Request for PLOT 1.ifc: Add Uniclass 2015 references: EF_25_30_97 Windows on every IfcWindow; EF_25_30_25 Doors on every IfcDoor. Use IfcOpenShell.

First a look at what the model holds.

```python
import ifcopenshell

model = ifcopenshell.open("PLOT 1.ifc")
print(model.schema)
print("classifications:", [c.Name for c in model.by_type("IfcClassification")])
for ifc_class in ("IfcDoor", "IfcRoof", "IfcStair", "IfcWall", "IfcWindow"):
    print(ifc_class, len(model.by_type(ifc_class)))
```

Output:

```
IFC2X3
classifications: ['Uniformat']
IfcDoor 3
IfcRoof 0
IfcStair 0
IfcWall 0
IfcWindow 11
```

```python
import ifcopenshell
import ifcopenshell.api.classification

model = ifcopenshell.open("PLOT 1.ifc")

# IFC2X3 requires Source and Edition and has no link from the project to the system.
system = model.create_entity("IfcClassification", Source="NBS", Edition="2015", Name="Uniclass 2015")

codes = {
    "IfcWindow": ("EF_25_30_97", "Windows"),
    "IfcDoor": ("EF_25_30_25", "Doors"),
}
for ifc_class, (code, name) in codes.items():
    products = model.by_type(ifc_class)
    ifcopenshell.api.classification.add_reference(
        model, products=products, classification=system, identification=code, name=name
    )
    print(code, len(products))

model.write("PLOT 1-out.ifc")
```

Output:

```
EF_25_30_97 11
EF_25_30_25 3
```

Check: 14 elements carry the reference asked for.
